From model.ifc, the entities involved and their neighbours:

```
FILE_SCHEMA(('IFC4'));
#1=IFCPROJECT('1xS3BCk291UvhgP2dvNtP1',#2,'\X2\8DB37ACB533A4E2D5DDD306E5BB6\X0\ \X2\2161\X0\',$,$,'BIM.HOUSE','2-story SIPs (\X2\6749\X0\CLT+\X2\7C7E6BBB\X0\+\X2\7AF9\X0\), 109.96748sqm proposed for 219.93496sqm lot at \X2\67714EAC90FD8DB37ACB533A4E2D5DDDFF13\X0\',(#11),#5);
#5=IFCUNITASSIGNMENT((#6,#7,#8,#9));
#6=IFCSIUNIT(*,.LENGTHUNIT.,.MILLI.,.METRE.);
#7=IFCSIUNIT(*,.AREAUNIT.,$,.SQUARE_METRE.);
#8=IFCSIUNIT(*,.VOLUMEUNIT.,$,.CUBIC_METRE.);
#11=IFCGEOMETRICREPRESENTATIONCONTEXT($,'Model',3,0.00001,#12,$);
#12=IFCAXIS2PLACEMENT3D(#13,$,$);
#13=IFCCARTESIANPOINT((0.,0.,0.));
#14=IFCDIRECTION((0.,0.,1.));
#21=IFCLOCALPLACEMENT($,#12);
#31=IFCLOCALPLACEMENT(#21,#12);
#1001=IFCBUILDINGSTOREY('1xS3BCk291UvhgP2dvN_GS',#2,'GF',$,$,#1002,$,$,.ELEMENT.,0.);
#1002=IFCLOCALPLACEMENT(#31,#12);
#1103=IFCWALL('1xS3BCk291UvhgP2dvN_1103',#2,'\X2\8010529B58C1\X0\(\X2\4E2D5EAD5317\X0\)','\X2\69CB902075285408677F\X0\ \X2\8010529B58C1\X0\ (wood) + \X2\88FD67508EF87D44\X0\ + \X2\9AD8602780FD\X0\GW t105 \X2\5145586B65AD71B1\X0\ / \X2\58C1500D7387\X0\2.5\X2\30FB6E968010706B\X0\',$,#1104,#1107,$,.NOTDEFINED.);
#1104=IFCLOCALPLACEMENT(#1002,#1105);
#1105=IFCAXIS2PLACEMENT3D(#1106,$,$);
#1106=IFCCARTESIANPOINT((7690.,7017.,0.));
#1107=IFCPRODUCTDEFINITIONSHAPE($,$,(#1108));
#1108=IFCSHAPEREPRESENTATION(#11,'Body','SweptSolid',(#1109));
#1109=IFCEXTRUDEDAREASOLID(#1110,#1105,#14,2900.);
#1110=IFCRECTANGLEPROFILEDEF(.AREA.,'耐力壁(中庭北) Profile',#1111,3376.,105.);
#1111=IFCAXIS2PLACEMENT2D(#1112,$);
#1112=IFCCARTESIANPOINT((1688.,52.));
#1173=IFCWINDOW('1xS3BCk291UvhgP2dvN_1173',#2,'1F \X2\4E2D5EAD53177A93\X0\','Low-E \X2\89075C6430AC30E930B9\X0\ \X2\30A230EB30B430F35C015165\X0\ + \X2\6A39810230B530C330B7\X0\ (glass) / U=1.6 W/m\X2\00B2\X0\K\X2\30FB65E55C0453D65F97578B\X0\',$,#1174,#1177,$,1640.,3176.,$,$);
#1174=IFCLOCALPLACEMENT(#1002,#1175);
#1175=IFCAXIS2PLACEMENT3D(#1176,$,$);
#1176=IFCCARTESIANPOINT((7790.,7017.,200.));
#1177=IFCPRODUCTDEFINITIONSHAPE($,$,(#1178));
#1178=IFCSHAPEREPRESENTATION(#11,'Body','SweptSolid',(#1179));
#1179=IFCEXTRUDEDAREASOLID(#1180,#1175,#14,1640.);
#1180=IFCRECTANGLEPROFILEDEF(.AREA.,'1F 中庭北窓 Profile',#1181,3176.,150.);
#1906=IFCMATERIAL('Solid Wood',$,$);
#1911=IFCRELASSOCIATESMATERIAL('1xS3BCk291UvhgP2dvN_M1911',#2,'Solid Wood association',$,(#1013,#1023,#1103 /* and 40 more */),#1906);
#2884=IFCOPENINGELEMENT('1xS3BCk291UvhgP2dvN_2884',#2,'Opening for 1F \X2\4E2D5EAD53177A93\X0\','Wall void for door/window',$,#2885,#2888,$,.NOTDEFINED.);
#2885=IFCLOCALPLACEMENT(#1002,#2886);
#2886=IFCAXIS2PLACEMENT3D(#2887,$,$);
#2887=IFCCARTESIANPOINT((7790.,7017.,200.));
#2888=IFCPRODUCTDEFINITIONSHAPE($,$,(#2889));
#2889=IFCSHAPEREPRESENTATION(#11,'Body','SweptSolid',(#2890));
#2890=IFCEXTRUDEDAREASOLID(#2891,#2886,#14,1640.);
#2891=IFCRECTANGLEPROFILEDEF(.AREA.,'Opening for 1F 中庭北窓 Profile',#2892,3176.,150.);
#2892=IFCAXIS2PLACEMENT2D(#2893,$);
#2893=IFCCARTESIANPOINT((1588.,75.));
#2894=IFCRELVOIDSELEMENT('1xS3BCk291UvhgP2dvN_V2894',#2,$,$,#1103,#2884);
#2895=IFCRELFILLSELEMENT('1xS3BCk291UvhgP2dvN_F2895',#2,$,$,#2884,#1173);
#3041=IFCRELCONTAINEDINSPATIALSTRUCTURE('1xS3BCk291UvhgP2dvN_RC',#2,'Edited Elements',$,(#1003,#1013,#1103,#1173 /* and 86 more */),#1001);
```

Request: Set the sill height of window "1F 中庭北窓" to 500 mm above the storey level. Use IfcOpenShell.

```python
import numpy as np
import ifcopenshell
import ifcopenshell.api.geometry
import ifcopenshell.geom
import ifcopenshell.util.element
import ifcopenshell.util.placement
import ifcopenshell.util.shape
import ifcopenshell.util.unit

model = ifcopenshell.open("model.ifc")
unit_scale = ifcopenshell.util.unit.calculate_unit_scale(model)

window = model.by_id(1173)
opening = window.FillsVoids[0].RelatingOpeningElement
storey = ifcopenshell.util.element.get_container(window, ifc_class="IfcBuildingStorey")
level = ifcopenshell.util.placement.get_local_placement(storey.ObjectPlacement)[2, 3]

# The opening's origin need not be at the sill, so measure its lowest point.
shape = ifcopenshell.geom.create_shape(ifcopenshell.geom.settings(), opening)
bottom = ifcopenshell.util.shape.get_shape_bottom_elevation(shape, shape.geometry) / unit_scale
dz = level + 0.5 / unit_scale - bottom

shift = np.array([0.0, 0.0, dz])
# The window is not placed relative to its opening, so move both.
for product in (opening, window):
    matrix = ifcopenshell.util.placement.get_local_placement(product.ObjectPlacement)
    matrix[:3, 3] += shift
    ifcopenshell.api.geometry.edit_object_placement(model, product=product, matrix=matrix, is_si=False)

print(f"moved by {dz * unit_scale:+.3f} m")

model.write("model-out.ifc")
```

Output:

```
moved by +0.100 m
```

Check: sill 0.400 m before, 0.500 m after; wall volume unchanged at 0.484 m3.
